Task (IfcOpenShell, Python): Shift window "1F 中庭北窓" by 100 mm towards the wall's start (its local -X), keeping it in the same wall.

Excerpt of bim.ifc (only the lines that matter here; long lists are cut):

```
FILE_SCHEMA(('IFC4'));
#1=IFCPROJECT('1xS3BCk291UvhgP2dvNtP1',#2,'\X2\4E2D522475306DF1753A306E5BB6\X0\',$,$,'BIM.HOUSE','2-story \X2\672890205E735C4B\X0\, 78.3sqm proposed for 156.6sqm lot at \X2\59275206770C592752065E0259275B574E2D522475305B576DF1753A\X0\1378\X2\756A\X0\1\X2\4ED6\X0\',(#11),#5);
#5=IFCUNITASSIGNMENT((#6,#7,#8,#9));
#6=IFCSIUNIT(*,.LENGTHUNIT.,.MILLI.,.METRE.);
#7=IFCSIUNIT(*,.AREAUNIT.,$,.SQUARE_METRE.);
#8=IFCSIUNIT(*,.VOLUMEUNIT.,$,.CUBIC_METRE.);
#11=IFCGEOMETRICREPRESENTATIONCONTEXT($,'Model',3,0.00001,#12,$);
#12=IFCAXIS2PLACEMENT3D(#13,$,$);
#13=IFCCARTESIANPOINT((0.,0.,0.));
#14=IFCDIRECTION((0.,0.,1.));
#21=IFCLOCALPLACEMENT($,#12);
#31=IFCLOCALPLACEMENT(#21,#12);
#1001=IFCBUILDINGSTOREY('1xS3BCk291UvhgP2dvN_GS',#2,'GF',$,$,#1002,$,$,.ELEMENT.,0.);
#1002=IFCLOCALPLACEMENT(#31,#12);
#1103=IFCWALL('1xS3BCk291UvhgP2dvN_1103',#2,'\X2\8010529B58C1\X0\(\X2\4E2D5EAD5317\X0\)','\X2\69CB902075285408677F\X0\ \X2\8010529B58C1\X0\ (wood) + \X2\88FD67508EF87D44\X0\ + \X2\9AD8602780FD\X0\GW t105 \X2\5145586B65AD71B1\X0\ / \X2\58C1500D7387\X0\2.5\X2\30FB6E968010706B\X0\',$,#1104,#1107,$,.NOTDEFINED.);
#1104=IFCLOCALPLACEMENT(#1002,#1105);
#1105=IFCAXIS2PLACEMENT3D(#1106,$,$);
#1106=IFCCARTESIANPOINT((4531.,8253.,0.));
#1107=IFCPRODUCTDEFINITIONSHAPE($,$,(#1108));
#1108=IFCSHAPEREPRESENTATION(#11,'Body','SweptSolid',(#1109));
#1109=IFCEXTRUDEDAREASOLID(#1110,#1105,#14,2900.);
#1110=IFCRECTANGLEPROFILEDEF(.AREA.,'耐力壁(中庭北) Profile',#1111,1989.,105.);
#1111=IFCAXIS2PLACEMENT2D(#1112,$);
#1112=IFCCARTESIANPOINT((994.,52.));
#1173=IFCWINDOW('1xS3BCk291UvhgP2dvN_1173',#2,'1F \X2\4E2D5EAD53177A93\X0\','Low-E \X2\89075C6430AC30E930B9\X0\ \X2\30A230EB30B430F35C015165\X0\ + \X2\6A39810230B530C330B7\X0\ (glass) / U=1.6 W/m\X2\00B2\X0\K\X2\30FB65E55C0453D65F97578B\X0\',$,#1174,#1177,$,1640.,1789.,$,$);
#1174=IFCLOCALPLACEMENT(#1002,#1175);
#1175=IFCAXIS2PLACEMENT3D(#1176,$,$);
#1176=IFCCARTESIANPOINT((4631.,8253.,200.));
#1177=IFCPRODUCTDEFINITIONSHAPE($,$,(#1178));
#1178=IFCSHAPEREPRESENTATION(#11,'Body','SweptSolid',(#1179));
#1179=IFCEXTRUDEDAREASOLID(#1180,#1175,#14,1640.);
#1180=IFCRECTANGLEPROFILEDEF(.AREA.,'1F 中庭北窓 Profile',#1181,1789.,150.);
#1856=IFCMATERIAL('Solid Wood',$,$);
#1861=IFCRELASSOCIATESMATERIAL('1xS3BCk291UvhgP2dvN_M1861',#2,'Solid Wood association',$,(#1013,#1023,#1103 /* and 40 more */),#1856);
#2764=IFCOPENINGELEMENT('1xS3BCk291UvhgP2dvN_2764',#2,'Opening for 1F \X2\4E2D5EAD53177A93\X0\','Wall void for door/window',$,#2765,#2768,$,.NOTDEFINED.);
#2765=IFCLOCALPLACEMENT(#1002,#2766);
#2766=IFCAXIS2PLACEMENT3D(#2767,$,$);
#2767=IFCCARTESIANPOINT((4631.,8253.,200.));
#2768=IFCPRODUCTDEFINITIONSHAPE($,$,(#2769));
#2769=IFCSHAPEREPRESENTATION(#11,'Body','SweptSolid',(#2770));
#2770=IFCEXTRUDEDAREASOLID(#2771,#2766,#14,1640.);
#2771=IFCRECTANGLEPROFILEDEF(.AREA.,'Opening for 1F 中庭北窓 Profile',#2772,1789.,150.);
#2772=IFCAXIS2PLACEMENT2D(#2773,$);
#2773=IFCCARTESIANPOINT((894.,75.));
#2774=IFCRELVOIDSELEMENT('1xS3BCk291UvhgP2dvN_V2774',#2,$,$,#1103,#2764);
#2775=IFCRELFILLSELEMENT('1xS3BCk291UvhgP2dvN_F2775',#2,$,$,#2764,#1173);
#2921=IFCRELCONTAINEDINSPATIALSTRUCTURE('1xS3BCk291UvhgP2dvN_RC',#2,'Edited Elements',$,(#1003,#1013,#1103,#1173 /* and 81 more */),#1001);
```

```python
import ifcopenshell
import ifcopenshell.api.geometry
import ifcopenshell.util.placement

model = ifcopenshell.open("bim.ifc")

window = model.by_guid("1xS3BCk291UvhgP2dvN_1173")
opening = window.FillsVoids[0].RelatingOpeningElement
wall = opening.VoidsElements[0].RelatingBuildingElement

wall_matrix = ifcopenshell.util.placement.get_local_placement(wall.ObjectPlacement)
shift = wall_matrix[:3, 0] * -100.0
before = ifcopenshell.util.placement.get_local_placement(window.ObjectPlacement)[:3, 3].copy()

# The window is not placed relative to its opening, so move both.
for product in (opening, window):
    matrix = ifcopenshell.util.placement.get_local_placement(product.ObjectPlacement)
    matrix[:3, 3] += shift
    ifcopenshell.api.geometry.edit_object_placement(model, product=product, matrix=matrix, is_si=False)

after = ifcopenshell.util.placement.get_local_placement(window.ObjectPlacement)[:3, 3]
print("window moved by", (after - before).round(3) + 0.0)

model.write("bim_v2.ifc")
```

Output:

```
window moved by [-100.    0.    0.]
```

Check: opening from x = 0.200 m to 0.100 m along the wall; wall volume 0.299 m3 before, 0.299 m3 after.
